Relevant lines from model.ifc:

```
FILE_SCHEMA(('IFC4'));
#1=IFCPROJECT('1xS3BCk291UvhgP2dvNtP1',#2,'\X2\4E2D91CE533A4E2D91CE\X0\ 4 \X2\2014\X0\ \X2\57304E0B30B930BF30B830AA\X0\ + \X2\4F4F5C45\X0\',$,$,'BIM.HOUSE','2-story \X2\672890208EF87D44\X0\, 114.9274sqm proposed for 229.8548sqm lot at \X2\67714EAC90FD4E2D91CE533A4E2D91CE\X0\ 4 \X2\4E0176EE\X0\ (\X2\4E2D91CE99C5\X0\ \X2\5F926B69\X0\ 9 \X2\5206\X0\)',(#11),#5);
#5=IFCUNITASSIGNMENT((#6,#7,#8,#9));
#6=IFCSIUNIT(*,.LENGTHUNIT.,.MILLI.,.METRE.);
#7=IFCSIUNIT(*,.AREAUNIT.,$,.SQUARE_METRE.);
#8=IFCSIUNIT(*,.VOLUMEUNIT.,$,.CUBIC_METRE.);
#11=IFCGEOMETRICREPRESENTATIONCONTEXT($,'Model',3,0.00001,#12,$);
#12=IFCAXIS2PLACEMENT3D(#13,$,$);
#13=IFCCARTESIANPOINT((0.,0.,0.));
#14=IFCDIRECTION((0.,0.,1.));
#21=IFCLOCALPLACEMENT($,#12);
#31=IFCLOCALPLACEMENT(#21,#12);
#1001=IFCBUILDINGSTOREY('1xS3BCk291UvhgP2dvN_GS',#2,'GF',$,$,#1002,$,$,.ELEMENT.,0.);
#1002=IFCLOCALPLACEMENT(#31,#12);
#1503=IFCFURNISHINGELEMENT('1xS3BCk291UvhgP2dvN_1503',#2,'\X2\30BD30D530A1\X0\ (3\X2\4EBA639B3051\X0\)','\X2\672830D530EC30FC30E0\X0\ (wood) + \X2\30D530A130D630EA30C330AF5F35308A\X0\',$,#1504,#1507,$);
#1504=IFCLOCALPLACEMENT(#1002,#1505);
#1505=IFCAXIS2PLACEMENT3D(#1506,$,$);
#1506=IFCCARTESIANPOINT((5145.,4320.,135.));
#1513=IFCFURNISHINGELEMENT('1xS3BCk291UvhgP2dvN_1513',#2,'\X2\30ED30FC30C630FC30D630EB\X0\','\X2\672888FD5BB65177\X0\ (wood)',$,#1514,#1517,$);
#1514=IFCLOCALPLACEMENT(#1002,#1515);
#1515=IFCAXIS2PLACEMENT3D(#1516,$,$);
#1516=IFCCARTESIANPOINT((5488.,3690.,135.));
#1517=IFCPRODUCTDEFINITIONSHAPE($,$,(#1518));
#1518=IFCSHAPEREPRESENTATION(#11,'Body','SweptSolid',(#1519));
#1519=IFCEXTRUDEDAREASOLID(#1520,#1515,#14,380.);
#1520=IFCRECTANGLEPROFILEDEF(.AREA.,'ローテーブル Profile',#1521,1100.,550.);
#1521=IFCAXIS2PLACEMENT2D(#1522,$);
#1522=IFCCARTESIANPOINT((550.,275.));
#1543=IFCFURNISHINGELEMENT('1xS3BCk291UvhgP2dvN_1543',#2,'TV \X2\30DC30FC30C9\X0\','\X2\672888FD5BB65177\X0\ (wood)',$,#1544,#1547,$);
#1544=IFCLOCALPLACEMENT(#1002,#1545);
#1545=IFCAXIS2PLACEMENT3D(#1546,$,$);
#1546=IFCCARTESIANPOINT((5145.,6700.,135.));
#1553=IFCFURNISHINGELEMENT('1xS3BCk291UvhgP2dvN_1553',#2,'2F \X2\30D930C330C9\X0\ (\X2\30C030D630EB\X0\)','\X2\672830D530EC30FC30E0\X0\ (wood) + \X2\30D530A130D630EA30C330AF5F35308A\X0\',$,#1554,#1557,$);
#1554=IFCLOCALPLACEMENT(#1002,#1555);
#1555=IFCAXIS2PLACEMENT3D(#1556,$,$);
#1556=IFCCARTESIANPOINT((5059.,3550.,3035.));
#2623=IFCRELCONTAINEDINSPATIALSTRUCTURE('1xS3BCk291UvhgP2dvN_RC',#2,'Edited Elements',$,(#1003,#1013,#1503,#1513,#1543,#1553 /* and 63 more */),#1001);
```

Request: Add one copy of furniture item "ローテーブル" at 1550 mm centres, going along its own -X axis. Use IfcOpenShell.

```python
import ifcopenshell
import ifcopenshell.api.geometry
import ifcopenshell.api.root
import ifcopenshell.util.element
import ifcopenshell.util.placement
import ifcopenshell.util.unit

model = ifcopenshell.open("model.ifc")
unit_scale = ifcopenshell.util.unit.calculate_unit_scale(model)


def reuse_history(source, copy):
    """copy_class also copies each property set's owner history, people and application; keep the originals."""
    for rel in copy.IsDefinedBy:
        if rel.is_a("IfcRelDefinesByProperties") and (history := rel.RelatingPropertyDefinition.OwnerHistory):
            rel.RelatingPropertyDefinition.OwnerHistory = source.OwnerHistory
            ifcopenshell.util.element.remove_deep2(model, history)


source = model.by_guid("1xS3BCk291UvhgP2dvN_1513")
base = ifcopenshell.util.placement.get_local_placement(source.ObjectPlacement)
step = -base[:3, 0] * 1.55 / unit_scale

for i in range(1, 2):
    copy = ifcopenshell.api.root.copy_class(model, product=source)
    copy.Representation = ifcopenshell.util.element.copy_deep(
        model, source.Representation, exclude=["IfcGeometricRepresentationContext", "IfcRepresentationMap"]
    )
    reuse_history(source, copy)
    matrix = base.copy()
    matrix[:3, 3] += i * step
    print("added at", matrix[:3, 3].round(3) + 0.0)
    ifcopenshell.api.geometry.edit_object_placement(model, product=copy, matrix=matrix, is_si=False)

model.write("model-out.ifc")
```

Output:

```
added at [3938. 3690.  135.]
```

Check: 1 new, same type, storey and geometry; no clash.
